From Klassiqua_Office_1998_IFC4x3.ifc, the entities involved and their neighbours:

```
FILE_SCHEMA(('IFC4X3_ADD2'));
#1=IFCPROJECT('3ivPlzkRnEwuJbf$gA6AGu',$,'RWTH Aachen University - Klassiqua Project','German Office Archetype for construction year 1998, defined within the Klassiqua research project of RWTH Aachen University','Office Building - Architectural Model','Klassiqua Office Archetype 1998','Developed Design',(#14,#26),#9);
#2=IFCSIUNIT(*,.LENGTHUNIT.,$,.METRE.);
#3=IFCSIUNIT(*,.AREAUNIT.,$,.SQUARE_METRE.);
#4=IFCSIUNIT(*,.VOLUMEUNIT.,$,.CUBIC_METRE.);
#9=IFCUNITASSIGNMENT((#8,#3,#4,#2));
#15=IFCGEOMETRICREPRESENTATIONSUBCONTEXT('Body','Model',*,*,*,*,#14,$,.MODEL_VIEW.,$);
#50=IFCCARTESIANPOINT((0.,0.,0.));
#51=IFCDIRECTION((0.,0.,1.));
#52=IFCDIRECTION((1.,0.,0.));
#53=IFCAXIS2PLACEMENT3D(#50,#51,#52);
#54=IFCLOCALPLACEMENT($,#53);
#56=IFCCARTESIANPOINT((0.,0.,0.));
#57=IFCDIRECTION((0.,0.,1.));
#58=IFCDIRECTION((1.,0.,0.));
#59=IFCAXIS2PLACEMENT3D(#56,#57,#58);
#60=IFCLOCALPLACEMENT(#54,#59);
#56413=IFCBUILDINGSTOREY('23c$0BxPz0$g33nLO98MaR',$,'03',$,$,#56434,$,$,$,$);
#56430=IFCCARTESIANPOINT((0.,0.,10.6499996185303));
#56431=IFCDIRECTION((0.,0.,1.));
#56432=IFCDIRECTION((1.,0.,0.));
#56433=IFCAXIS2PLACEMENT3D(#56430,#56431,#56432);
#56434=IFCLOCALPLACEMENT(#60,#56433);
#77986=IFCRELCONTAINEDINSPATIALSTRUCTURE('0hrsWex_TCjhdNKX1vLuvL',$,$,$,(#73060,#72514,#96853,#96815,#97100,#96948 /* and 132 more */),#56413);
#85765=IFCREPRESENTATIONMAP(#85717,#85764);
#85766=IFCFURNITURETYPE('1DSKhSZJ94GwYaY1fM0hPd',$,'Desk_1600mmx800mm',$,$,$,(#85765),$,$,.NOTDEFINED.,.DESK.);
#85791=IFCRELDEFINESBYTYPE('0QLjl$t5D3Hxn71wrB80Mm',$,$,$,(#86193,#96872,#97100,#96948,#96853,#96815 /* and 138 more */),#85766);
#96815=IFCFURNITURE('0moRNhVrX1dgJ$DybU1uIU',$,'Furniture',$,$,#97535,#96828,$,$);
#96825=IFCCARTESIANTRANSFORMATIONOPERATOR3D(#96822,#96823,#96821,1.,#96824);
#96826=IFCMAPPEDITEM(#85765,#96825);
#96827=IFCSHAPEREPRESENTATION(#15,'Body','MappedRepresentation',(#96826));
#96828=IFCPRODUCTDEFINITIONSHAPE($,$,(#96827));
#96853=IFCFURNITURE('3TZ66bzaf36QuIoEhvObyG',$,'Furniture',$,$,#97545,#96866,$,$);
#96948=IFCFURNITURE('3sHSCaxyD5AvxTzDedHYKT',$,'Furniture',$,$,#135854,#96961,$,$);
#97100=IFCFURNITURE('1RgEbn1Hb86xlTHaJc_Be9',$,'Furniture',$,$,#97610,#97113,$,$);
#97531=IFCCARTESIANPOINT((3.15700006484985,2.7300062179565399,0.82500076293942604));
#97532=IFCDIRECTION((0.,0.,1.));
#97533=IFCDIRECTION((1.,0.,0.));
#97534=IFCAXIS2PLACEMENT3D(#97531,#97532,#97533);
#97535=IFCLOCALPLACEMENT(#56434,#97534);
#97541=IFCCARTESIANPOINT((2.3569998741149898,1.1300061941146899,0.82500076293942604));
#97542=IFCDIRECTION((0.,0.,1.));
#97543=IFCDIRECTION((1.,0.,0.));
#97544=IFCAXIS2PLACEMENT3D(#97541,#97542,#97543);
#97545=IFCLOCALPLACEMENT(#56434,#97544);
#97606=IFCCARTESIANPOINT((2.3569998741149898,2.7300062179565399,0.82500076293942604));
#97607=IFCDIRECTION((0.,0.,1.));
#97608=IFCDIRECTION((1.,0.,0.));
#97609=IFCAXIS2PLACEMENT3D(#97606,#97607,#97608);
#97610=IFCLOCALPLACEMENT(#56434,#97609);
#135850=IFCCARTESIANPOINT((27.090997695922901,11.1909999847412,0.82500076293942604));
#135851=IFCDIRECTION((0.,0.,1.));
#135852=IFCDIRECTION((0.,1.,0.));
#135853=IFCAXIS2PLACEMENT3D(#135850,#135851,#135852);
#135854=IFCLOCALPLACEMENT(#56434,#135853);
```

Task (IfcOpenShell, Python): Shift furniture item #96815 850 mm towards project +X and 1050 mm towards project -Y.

```python
import ifcopenshell
import ifcopenshell.api.geometry
import ifcopenshell.util.placement
import ifcopenshell.util.unit

model = ifcopenshell.open("Klassiqua_Office_1998_IFC4x3.ifc")
unit_scale = ifcopenshell.util.unit.calculate_unit_scale(model)

item = model.by_guid("0moRNhVrX1dgJ$DybU1uIU")
matrix = ifcopenshell.util.placement.get_local_placement(item.ObjectPlacement)
matrix[0, 3] += 0.85 / unit_scale
matrix[1, 3] -= 1.05 / unit_scale
ifcopenshell.api.geometry.edit_object_placement(model, product=item, matrix=matrix, is_si=False)

print(ifcopenshell.util.placement.get_local_placement(item.ObjectPlacement).round(3) + 0.0)

model.write("Klassiqua_Office_1998_IFC4x3_updated.ifc")
```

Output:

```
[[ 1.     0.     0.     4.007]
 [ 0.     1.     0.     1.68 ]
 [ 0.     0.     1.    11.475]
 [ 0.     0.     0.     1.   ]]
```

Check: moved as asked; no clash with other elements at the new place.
